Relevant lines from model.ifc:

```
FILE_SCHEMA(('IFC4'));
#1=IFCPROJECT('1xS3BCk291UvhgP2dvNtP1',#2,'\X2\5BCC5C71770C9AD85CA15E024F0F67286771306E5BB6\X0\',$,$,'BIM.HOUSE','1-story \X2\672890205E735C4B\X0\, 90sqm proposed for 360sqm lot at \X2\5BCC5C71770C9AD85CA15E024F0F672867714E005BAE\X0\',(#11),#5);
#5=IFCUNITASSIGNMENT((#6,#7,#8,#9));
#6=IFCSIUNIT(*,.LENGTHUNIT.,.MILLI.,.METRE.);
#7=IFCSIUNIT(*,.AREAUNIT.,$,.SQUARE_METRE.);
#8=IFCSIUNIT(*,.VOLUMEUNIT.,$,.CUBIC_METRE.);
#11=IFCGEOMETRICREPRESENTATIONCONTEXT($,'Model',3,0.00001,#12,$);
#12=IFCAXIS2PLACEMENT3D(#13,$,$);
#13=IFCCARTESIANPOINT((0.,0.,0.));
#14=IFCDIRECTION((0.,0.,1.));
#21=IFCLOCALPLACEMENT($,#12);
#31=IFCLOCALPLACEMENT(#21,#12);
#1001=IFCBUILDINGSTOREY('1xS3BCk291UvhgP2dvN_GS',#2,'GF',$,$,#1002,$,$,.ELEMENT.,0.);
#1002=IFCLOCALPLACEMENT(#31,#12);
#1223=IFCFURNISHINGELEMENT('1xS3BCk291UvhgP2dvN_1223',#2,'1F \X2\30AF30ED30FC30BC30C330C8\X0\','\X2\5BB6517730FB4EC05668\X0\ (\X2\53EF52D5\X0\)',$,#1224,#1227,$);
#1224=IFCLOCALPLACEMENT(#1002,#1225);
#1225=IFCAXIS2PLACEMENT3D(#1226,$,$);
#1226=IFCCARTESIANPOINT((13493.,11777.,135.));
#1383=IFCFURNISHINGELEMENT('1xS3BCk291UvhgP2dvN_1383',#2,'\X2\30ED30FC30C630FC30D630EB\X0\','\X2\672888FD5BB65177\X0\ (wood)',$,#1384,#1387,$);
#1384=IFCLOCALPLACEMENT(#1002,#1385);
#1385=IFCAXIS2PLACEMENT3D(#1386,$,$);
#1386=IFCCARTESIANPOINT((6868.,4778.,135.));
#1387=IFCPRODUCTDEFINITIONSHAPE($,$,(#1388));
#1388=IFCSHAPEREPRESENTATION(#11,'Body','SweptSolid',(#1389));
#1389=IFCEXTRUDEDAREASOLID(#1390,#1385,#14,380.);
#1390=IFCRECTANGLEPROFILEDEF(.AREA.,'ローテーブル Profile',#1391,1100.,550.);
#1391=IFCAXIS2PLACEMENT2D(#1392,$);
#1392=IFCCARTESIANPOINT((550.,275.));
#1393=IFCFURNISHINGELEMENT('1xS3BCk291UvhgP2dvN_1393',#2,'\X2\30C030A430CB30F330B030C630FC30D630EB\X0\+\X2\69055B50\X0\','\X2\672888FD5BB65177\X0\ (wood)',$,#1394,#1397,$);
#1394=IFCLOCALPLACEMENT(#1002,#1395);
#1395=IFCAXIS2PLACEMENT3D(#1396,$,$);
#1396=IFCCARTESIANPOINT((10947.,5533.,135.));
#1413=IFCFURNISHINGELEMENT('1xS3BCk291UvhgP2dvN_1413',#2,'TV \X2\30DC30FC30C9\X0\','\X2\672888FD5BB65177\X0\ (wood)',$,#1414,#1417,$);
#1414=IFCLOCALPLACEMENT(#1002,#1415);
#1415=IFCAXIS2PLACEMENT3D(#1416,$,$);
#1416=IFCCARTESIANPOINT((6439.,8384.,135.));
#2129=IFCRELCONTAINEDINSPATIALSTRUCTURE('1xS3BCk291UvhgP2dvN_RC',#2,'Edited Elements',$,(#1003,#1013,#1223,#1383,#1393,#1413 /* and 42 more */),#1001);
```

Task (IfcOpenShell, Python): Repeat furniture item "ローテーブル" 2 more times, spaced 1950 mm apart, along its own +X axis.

```python
import ifcopenshell
import ifcopenshell.api.geometry
import ifcopenshell.api.root
import ifcopenshell.util.element
import ifcopenshell.util.placement
import ifcopenshell.util.unit

model = ifcopenshell.open("model.ifc")
unit_scale = ifcopenshell.util.unit.calculate_unit_scale(model)


def reuse_history(source, copy):
    """copy_class also copies each property set's owner history, people and application; keep the originals."""
    for rel in copy.IsDefinedBy:
        if rel.is_a("IfcRelDefinesByProperties") and (history := rel.RelatingPropertyDefinition.OwnerHistory):
            rel.RelatingPropertyDefinition.OwnerHistory = source.OwnerHistory
            ifcopenshell.util.element.remove_deep2(model, history)


source = model.by_guid("1xS3BCk291UvhgP2dvN_1383")
base = ifcopenshell.util.placement.get_local_placement(source.ObjectPlacement)
step = base[:3, 0] * 1.95 / unit_scale

for i in range(1, 3):
    copy = ifcopenshell.api.root.copy_class(model, product=source)
    copy.Representation = ifcopenshell.util.element.copy_deep(
        model, source.Representation, exclude=["IfcGeometricRepresentationContext", "IfcRepresentationMap"]
    )
    reuse_history(source, copy)
    matrix = base.copy()
    matrix[:3, 3] += i * step
    print("added at", matrix[:3, 3].round(3) + 0.0)
    ifcopenshell.api.geometry.edit_object_placement(model, product=copy, matrix=matrix, is_si=False)

model.write("model_updated.ifc")
```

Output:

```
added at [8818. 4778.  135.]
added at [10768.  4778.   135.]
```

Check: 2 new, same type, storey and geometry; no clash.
